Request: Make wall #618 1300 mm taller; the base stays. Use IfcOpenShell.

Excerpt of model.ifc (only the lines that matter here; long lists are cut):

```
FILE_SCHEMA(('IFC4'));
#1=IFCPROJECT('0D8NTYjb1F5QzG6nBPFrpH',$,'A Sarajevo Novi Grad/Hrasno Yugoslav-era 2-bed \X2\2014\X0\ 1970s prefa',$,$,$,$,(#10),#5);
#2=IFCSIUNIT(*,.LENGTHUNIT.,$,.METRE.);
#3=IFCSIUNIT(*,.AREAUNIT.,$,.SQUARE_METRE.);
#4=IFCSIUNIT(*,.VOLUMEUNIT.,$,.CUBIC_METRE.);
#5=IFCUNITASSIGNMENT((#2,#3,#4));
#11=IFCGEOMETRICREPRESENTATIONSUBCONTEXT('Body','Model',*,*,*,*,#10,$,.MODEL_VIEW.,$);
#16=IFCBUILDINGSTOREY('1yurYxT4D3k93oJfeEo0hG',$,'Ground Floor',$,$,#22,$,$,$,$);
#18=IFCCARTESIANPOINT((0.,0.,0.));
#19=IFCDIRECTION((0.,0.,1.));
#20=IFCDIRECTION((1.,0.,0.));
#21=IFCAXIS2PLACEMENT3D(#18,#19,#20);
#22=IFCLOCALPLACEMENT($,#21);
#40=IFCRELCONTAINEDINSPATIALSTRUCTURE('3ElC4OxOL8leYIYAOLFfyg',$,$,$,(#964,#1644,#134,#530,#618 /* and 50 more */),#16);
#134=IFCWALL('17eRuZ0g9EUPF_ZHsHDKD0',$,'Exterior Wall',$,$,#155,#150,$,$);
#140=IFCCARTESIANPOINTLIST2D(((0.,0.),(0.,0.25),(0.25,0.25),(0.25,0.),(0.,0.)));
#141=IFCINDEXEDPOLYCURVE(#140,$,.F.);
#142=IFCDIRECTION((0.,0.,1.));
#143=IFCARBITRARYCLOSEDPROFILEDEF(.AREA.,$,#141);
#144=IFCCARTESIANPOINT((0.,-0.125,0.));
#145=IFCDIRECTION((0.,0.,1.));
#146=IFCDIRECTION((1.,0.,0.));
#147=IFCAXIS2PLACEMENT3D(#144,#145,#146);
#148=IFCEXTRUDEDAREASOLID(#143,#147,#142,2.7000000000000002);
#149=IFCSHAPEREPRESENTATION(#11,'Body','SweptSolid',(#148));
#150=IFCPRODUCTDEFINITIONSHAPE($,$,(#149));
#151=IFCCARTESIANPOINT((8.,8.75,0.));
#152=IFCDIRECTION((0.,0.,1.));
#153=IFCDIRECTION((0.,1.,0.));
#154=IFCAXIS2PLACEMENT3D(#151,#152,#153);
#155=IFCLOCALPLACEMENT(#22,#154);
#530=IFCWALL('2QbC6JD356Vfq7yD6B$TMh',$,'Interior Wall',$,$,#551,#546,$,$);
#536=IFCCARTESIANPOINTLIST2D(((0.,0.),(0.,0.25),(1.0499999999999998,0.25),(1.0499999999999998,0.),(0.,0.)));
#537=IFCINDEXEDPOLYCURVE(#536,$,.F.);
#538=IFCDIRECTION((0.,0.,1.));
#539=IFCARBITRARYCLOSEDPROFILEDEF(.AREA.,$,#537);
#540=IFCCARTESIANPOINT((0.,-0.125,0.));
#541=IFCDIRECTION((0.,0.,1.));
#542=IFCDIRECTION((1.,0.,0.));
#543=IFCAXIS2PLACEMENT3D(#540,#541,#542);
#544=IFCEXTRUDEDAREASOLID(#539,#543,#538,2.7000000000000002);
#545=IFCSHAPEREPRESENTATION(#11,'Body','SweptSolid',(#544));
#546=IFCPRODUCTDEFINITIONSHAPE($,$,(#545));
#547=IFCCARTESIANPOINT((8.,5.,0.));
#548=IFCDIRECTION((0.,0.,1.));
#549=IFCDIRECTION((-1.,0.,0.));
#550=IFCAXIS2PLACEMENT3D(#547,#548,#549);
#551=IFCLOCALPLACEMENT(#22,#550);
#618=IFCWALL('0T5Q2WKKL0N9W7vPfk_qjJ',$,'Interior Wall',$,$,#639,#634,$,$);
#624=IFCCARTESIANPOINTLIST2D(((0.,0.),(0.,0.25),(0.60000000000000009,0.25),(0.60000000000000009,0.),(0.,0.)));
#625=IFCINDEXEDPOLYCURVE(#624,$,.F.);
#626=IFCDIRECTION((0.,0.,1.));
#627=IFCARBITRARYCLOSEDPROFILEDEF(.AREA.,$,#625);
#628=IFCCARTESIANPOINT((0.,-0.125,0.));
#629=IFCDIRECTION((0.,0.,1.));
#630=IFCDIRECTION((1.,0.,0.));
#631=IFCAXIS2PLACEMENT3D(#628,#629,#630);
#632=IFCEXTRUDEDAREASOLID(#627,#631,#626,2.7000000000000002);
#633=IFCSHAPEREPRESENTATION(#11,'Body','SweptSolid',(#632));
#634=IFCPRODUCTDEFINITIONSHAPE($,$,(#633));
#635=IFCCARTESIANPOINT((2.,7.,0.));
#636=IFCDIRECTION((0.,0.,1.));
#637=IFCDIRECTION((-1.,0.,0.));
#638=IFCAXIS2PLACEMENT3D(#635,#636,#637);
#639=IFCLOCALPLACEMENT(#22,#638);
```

```python
import ifcopenshell
import ifcopenshell.geom
import ifcopenshell.util.representation
import ifcopenshell.util.shape
import ifcopenshell.util.unit

model = ifcopenshell.open("model.ifc")
unit_scale = ifcopenshell.util.unit.calculate_unit_scale(model)
settings = ifcopenshell.geom.settings()


def volume(element):
    """Net volume in cubic metres, openings subtracted."""
    shape = ifcopenshell.geom.create_shape(settings, element)
    return ifcopenshell.util.shape.get_volume(shape.geometry)


wall = model.by_guid("0T5Q2WKKL0N9W7vPfk_qjJ")
before = volume(wall)

body = ifcopenshell.util.representation.get_representation(wall, "Model", "Body")
solid = body.Items[0]
old_height = solid.Depth
solid.Depth += 1.3 / unit_scale
after = volume(wall)

print(f"height {old_height:g} -> {solid.Depth:g}, volume {before:.3f} -> {after:.3f} m3")

model.write("model_v2.ifc")
```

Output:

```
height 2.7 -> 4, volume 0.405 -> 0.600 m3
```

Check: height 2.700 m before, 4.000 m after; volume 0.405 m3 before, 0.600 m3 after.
